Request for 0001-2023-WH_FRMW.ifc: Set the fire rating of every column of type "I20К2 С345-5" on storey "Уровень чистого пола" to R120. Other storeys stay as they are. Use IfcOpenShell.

First a look at what the model holds.

```python
import ifcopenshell
import ifcopenshell.util.element

model = ifcopenshell.open("0001-2023-WH_FRMW.ifc")
print(model.schema)
storey = next(s for s in model.by_type("IfcBuildingStorey") if s.Name == "Уровень чистого пола")
columns = [e for e in ifcopenshell.util.element.get_decomposition(storey) if e.is_a("IfcColumn")]
seen = {}
for e in columns:
    element_type = ifcopenshell.util.element.get_type(e)
    key = (element_type.Name if element_type != e and element_type else None, ifcopenshell.util.element.get_pset(e, "Pset_ColumnCommon", "FireRating"))
    seen[key] = seen.get(key, 0) + 1
for (name, value), count in sorted(seen.items(), key=str):
    print(count, "x", name, "|", value)
```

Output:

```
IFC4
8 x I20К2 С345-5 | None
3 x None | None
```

```python
import ifcopenshell
import ifcopenshell.api.pset
import ifcopenshell.util.element

model = ifcopenshell.open("0001-2023-WH_FRMW.ifc")

storey = next(s for s in model.by_type("IfcBuildingStorey") if s.Name == "Уровень чистого пола")
columns = [e for e in ifcopenshell.util.element.get_decomposition(storey) if e.is_a("IfcColumn")]

count = 0
for e in columns:
    element_type = ifcopenshell.util.element.get_type(e)
    if element_type in (None, e) or element_type.Name != "I20К2 С345-5":
        continue
    # add_pset returns the element's existing set when there is one.
    pset = ifcopenshell.api.pset.add_pset(model, product=e, name="Pset_ColumnCommon")
    ifcopenshell.api.pset.edit_pset(model, pset=pset, properties={"FireRating": "R120"})
    count += 1

print(count, "columns updated")

model.write("0001-2023-WH_FRMW_rev.ifc")
```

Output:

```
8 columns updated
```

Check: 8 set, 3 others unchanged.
